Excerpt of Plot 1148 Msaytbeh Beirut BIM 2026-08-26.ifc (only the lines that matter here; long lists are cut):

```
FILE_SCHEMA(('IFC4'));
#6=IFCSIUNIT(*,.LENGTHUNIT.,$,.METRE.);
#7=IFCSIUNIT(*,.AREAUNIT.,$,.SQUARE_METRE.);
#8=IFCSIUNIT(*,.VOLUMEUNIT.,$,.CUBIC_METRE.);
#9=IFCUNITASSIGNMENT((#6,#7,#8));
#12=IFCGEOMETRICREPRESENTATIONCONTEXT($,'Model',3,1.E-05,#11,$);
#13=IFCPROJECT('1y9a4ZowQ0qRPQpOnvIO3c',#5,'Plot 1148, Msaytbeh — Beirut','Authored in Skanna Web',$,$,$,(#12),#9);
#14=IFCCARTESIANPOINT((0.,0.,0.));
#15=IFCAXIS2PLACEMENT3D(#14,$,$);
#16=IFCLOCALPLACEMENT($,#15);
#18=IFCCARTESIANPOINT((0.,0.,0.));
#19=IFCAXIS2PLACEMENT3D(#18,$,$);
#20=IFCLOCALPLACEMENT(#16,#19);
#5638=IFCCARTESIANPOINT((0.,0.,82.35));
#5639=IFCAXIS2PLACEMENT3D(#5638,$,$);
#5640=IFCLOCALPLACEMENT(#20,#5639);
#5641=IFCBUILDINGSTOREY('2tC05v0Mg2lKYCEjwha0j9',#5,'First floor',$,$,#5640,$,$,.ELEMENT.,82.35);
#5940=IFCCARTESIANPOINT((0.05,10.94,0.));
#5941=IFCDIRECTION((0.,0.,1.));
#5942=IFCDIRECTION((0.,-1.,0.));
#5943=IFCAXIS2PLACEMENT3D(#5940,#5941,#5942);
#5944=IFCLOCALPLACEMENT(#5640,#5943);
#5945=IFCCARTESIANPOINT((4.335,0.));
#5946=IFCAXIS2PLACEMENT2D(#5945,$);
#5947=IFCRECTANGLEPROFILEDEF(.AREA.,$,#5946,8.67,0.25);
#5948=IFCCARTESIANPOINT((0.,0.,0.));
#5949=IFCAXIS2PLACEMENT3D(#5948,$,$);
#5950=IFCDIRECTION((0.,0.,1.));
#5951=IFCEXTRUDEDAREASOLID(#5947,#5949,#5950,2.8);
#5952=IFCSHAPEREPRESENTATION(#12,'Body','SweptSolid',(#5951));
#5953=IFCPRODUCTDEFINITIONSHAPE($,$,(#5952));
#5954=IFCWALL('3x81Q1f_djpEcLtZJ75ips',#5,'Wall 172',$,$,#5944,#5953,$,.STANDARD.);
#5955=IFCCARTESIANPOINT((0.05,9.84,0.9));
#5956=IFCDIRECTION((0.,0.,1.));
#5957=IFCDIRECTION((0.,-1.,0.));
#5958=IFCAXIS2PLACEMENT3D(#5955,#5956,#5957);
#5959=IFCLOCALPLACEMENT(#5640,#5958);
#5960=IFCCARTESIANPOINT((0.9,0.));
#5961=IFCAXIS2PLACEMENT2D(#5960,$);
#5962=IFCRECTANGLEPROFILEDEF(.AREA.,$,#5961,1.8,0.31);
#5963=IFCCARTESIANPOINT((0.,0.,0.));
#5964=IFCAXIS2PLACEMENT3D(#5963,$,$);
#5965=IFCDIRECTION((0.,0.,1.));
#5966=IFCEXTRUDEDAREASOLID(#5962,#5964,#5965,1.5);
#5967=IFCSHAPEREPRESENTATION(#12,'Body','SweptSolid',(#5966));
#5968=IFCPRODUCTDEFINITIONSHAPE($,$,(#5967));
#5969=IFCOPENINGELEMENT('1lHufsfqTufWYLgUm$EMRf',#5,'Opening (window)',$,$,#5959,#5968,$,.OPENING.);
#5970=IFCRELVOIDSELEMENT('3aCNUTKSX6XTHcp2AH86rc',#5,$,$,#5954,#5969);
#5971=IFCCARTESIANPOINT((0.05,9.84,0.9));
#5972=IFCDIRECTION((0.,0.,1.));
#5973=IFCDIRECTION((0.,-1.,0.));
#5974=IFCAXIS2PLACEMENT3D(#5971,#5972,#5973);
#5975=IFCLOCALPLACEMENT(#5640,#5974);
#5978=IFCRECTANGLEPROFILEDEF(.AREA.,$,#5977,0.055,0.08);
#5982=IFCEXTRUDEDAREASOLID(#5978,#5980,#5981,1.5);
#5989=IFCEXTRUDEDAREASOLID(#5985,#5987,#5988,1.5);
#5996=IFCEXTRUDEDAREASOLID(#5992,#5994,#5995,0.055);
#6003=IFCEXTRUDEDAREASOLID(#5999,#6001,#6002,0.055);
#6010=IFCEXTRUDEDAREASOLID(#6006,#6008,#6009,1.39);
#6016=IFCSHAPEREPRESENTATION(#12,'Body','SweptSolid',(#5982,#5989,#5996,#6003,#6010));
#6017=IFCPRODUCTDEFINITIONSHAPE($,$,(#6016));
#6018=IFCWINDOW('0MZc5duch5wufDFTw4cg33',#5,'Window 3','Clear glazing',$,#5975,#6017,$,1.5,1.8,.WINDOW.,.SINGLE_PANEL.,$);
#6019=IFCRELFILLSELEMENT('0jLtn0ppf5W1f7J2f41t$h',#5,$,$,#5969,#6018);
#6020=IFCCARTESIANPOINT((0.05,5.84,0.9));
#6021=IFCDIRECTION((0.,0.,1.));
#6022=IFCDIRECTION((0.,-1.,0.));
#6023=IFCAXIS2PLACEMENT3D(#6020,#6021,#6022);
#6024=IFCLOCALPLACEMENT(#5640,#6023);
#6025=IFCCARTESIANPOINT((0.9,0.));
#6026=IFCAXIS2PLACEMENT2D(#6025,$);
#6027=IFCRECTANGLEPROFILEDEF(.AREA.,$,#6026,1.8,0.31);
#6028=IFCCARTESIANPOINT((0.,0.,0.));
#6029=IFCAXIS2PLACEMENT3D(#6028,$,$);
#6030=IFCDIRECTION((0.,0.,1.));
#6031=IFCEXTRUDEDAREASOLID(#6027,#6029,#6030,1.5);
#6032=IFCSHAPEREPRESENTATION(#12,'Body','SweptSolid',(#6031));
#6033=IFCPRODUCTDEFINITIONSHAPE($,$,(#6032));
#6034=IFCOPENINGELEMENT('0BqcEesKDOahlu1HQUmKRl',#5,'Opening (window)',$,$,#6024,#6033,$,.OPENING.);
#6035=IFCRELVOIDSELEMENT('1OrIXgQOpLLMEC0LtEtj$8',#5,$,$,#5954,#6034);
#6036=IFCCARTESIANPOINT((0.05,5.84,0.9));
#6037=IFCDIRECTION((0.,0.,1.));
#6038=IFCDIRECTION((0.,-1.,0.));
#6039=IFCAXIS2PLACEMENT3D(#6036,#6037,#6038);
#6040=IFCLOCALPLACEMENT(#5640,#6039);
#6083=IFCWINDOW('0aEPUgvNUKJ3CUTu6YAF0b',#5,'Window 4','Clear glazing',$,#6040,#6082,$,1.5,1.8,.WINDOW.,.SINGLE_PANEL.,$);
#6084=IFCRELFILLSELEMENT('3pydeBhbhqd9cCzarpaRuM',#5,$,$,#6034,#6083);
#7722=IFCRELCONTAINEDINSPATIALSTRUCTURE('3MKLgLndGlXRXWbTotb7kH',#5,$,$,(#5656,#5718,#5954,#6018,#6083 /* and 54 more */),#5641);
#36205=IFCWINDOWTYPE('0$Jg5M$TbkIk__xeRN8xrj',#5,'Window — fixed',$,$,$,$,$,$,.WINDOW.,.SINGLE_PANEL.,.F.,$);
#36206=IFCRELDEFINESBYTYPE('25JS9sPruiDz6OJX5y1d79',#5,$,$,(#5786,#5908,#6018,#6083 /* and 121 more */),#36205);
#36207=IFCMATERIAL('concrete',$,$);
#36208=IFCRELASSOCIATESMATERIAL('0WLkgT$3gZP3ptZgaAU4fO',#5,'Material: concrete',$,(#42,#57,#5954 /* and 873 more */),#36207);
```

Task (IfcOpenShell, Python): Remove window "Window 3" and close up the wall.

```python
import ifcopenshell
import ifcopenshell.api.feature
import ifcopenshell.api.root
import ifcopenshell.geom
import ifcopenshell.util.shape

model = ifcopenshell.open("Plot 1148 Msaytbeh Beirut BIM 2026-08-26.ifc")
settings = ifcopenshell.geom.settings()


def volume(element):
    """Net volume in cubic metres, openings subtracted."""
    shape = ifcopenshell.geom.create_shape(settings, element)
    return ifcopenshell.util.shape.get_volume(shape.geometry)


window = model.by_guid("0MZc5duch5wufDFTw4cg33")
opening = window.FillsVoids[0].RelatingOpeningElement
wall = opening.VoidsElements[0].RelatingBuildingElement
before = volume(wall)

ifcopenshell.api.root.remove_product(model, product=window)
ifcopenshell.api.feature.remove_feature(model, feature=opening)

after = volume(wall)

print(f"wall volume {before:.3f} -> {after:.3f} m3")

model.write("Plot 1148 Msaytbeh Beirut BIM 2026-08-26_edited.ifc")
```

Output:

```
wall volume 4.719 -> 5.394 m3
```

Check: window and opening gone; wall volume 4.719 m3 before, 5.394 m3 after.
